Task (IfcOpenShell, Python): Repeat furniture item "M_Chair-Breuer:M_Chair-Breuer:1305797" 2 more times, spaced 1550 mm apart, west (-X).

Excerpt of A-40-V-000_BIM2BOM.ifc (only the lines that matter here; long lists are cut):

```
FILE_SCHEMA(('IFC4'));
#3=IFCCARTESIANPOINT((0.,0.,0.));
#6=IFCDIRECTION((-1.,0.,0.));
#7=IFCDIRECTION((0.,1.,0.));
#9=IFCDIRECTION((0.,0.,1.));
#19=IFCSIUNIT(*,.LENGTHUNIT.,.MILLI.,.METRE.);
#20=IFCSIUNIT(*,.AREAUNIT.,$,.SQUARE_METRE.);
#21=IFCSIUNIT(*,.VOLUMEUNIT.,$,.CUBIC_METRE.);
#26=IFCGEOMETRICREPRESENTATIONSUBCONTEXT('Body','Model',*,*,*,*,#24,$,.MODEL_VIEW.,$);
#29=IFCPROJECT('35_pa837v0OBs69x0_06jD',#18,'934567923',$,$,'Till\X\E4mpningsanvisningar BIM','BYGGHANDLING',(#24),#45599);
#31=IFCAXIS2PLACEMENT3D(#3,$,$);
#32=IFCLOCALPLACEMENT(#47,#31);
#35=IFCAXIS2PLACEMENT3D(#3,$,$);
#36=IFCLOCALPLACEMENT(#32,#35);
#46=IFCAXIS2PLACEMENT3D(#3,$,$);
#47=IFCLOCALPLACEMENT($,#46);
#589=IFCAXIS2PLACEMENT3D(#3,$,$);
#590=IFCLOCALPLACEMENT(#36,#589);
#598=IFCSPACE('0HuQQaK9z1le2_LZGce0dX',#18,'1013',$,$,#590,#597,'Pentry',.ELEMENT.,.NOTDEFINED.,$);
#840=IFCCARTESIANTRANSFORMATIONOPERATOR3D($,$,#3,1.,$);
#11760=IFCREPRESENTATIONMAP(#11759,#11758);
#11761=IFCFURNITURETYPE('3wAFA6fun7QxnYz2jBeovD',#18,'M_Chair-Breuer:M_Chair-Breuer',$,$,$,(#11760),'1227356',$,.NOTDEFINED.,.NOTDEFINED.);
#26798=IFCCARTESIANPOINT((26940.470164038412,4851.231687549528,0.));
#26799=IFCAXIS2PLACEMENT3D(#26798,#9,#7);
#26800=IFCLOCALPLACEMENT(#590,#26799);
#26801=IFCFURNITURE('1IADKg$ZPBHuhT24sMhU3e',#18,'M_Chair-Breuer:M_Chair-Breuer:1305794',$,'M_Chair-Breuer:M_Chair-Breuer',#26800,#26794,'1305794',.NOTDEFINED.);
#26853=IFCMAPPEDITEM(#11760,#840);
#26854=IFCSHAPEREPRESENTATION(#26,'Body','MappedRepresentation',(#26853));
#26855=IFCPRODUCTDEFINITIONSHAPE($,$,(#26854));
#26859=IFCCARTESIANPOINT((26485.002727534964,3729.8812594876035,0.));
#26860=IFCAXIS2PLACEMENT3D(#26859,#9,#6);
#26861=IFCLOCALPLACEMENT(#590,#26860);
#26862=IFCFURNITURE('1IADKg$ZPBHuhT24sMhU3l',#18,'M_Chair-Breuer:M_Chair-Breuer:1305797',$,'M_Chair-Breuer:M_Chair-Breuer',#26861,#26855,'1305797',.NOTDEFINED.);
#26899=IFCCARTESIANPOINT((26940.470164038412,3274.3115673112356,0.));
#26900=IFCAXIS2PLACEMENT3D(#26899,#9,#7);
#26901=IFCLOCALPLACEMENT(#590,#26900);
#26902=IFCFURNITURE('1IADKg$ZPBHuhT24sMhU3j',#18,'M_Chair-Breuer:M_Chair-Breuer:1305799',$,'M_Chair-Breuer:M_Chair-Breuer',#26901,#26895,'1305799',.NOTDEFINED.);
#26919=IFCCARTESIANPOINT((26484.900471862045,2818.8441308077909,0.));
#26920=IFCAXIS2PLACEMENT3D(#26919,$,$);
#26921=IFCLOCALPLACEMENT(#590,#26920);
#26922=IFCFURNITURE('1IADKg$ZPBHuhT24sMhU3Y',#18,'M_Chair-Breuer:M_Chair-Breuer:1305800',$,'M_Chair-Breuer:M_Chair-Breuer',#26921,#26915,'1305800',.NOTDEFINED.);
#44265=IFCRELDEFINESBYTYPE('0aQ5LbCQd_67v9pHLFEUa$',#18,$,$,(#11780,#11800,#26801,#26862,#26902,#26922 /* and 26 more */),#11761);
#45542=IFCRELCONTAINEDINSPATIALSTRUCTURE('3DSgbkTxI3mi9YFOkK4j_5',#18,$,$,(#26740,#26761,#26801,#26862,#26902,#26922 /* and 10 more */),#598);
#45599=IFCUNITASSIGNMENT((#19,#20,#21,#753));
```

```python
import numpy as np
import ifcopenshell
import ifcopenshell.api.geometry
import ifcopenshell.api.root
import ifcopenshell.util.element
import ifcopenshell.util.placement
import ifcopenshell.util.unit

model = ifcopenshell.open("A-40-V-000_BIM2BOM.ifc")
unit_scale = ifcopenshell.util.unit.calculate_unit_scale(model)


def reuse_history(source, copy):
    """copy_class also copies each property set's owner history, people and application; keep the originals."""
    for rel in copy.IsDefinedBy:
        if rel.is_a("IfcRelDefinesByProperties") and (history := rel.RelatingPropertyDefinition.OwnerHistory):
            rel.RelatingPropertyDefinition.OwnerHistory = source.OwnerHistory
            ifcopenshell.util.element.remove_deep2(model, history)


source = model.by_guid("1IADKg$ZPBHuhT24sMhU3l")
base = ifcopenshell.util.placement.get_local_placement(source.ObjectPlacement)
step = np.array([-1.0, 0.0, 0.0]) * 1.55 / unit_scale

for i in range(1, 3):
    copy = ifcopenshell.api.root.copy_class(model, product=source)
    copy.Representation = ifcopenshell.util.element.copy_deep(
        model, source.Representation, exclude=["IfcGeometricRepresentationContext", "IfcRepresentationMap"]
    )
    copy.Name = "M_Chair-Breuer:M_Chair-Breuer"
    copy.Tag = None
    reuse_history(source, copy)
    matrix = base.copy()
    matrix[:3, 3] += i * step
    print("added at", matrix[:3, 3].round(3) + 0.0)
    ifcopenshell.api.geometry.edit_object_placement(model, product=copy, matrix=matrix, is_si=False)

model.write("A-40-V-000_BIM2BOM_rev.ifc")
```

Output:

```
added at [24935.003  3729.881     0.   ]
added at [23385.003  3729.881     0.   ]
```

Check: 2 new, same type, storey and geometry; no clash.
